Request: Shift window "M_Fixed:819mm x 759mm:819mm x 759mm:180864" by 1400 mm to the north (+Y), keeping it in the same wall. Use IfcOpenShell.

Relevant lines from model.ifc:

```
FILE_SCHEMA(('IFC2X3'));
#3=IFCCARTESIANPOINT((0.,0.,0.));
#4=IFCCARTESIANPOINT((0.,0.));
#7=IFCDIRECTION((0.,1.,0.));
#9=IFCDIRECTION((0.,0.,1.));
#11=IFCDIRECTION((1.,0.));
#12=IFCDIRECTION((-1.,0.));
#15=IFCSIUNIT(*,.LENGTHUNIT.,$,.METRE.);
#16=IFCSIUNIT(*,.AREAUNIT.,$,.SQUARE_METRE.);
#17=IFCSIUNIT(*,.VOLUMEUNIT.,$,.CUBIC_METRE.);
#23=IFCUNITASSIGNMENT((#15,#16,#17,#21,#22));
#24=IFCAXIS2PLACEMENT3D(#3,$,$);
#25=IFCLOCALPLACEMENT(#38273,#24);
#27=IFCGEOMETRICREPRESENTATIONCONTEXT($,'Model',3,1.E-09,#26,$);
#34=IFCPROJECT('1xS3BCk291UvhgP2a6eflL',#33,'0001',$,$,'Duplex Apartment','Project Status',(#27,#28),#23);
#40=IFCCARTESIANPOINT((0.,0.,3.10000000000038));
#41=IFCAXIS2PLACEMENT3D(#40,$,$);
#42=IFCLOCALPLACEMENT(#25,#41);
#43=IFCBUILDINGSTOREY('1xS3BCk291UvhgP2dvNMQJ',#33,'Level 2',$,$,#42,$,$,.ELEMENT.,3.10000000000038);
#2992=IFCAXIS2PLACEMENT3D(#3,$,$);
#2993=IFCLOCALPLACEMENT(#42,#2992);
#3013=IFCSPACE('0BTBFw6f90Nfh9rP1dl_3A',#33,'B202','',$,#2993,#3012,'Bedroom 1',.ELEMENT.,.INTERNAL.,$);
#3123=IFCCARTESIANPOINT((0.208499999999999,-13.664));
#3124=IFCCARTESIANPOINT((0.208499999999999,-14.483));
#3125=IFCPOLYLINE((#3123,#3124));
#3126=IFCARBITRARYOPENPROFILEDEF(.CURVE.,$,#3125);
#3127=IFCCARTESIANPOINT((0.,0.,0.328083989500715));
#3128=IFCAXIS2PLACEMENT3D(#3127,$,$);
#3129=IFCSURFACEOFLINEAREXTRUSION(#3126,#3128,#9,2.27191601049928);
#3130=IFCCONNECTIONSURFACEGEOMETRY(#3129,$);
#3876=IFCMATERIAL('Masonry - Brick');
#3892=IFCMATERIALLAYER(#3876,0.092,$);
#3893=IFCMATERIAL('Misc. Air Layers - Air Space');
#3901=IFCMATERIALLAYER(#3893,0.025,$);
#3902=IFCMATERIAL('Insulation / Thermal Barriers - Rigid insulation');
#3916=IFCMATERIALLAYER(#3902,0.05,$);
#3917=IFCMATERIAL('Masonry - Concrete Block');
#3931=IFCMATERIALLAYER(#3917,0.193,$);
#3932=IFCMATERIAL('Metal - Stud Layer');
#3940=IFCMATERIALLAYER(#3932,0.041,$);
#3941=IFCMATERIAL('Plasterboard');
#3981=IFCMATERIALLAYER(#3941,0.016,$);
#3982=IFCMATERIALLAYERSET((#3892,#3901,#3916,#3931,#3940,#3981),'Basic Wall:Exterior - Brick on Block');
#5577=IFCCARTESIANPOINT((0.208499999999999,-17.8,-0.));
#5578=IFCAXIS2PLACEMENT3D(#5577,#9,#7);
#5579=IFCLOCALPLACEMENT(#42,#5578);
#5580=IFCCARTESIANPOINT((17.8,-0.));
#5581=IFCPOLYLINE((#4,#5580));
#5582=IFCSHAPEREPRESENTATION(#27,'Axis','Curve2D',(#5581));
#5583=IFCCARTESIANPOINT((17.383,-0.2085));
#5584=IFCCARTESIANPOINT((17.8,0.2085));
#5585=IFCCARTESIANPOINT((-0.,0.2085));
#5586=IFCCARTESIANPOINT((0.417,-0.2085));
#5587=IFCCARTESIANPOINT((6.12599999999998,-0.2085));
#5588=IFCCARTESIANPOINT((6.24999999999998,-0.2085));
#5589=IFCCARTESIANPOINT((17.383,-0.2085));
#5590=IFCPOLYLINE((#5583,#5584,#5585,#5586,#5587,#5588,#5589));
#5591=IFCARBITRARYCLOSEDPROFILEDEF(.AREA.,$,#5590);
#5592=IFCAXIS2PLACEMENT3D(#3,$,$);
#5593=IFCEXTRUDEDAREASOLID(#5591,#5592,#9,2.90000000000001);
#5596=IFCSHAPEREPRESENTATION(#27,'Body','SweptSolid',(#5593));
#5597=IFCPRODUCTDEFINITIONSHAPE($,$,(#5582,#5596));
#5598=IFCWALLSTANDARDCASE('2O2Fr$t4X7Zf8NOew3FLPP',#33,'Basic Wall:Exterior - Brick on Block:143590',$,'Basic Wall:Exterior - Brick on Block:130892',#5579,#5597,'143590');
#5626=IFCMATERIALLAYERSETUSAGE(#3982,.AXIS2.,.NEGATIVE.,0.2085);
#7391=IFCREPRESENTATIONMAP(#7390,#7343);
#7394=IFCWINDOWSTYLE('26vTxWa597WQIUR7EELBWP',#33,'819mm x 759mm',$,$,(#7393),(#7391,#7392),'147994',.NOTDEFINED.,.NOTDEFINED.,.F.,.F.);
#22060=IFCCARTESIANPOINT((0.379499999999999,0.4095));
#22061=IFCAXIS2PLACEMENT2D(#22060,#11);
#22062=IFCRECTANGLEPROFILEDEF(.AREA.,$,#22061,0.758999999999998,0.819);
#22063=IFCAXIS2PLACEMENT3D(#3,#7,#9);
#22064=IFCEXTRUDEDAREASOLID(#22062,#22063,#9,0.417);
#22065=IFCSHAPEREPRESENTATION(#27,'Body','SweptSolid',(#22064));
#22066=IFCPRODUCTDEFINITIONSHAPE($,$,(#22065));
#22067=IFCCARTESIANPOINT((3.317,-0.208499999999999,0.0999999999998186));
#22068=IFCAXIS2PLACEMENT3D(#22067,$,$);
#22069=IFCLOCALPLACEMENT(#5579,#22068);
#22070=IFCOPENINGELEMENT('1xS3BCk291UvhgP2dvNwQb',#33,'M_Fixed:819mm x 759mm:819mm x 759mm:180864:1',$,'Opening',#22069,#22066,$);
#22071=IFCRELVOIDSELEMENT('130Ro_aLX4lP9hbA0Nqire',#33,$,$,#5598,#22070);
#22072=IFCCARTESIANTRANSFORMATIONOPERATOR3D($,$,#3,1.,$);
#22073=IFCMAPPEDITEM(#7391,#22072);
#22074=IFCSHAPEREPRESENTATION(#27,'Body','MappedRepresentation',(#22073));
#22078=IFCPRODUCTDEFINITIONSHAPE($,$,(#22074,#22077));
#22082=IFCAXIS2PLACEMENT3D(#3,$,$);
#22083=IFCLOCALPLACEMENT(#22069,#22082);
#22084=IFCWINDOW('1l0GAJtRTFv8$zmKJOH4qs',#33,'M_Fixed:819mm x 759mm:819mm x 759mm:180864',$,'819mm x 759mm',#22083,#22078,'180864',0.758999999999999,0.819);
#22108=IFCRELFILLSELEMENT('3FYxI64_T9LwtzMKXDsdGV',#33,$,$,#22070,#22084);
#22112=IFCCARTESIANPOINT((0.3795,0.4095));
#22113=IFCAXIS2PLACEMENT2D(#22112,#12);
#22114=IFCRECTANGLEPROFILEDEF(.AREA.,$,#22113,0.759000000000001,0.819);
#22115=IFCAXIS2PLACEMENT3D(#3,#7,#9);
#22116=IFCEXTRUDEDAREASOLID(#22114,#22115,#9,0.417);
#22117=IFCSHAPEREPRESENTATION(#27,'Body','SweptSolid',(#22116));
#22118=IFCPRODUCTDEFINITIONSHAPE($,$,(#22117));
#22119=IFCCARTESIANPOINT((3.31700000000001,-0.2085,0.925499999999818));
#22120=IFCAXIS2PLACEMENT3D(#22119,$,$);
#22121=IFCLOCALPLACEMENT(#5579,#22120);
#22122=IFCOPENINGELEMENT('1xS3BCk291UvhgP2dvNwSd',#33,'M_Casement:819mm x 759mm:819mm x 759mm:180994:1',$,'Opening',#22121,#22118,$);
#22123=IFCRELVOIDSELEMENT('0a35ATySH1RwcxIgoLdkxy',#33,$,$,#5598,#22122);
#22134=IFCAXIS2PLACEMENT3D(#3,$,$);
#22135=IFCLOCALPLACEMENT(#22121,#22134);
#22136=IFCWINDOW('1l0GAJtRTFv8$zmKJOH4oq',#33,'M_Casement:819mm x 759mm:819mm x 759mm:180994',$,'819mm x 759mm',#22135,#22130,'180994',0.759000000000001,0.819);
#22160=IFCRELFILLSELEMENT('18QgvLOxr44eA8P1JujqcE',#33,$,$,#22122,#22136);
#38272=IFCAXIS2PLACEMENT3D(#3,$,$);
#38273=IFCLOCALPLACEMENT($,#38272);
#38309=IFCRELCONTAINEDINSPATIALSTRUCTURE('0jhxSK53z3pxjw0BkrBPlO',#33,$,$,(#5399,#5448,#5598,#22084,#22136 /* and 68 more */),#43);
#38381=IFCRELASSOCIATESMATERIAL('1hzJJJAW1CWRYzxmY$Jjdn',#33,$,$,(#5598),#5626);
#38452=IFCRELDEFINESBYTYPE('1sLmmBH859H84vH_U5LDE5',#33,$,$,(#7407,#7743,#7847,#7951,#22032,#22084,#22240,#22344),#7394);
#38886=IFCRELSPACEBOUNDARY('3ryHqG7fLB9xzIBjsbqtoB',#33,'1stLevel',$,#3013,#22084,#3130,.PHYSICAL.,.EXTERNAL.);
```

```python
import numpy as np
import ifcopenshell
import ifcopenshell.api.geometry
import ifcopenshell.util.placement
import ifcopenshell.util.unit

model = ifcopenshell.open("model.ifc")
unit_scale = ifcopenshell.util.unit.calculate_unit_scale(model)

window = model.by_guid("1l0GAJtRTFv8$zmKJOH4qs")
opening = window.FillsVoids[0].RelatingOpeningElement
wall = opening.VoidsElements[0].RelatingBuildingElement

wall_matrix = ifcopenshell.util.placement.get_local_placement(wall.ObjectPlacement)
shift = wall_matrix[:3, 0] * 1.4 / unit_scale
before = ifcopenshell.util.placement.get_local_placement(window.ObjectPlacement)[:3, 3].copy()

# The window is placed relative to its opening, so it follows when the opening moves.
matrix = ifcopenshell.util.placement.get_local_placement(opening.ObjectPlacement)
matrix[:3, 3] += shift
ifcopenshell.api.geometry.edit_object_placement(
    model, product=opening, matrix=matrix, is_si=False, should_transform_children=True
)

# Space boundary surfaces are stored in each space's coordinates; move them too.
for rel in window.ProvidesBoundaries:
    if not rel.ConnectionGeometry:
        continue
    surface = rel.ConnectionGeometry.SurfaceOnRelatingElement
    space_matrix = ifcopenshell.util.placement.get_local_placement(rel.RelatingSpace.ObjectPlacement)
    point = np.array(surface.Position.Location.Coordinates) + space_matrix[:3, :3].T @ shift
    surface.Position = model.createIfcAxis2Placement3D(
        model.createIfcCartesianPoint(point.tolist()), surface.Position.Axis, surface.Position.RefDirection
    )

after = ifcopenshell.util.placement.get_local_placement(window.ObjectPlacement)[:3, 3]
print("window moved by", (after - before).round(3) + 0.0)

model.write("model-out.ifc")
```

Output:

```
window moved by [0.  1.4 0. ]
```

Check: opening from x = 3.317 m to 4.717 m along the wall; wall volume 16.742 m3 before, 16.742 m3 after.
